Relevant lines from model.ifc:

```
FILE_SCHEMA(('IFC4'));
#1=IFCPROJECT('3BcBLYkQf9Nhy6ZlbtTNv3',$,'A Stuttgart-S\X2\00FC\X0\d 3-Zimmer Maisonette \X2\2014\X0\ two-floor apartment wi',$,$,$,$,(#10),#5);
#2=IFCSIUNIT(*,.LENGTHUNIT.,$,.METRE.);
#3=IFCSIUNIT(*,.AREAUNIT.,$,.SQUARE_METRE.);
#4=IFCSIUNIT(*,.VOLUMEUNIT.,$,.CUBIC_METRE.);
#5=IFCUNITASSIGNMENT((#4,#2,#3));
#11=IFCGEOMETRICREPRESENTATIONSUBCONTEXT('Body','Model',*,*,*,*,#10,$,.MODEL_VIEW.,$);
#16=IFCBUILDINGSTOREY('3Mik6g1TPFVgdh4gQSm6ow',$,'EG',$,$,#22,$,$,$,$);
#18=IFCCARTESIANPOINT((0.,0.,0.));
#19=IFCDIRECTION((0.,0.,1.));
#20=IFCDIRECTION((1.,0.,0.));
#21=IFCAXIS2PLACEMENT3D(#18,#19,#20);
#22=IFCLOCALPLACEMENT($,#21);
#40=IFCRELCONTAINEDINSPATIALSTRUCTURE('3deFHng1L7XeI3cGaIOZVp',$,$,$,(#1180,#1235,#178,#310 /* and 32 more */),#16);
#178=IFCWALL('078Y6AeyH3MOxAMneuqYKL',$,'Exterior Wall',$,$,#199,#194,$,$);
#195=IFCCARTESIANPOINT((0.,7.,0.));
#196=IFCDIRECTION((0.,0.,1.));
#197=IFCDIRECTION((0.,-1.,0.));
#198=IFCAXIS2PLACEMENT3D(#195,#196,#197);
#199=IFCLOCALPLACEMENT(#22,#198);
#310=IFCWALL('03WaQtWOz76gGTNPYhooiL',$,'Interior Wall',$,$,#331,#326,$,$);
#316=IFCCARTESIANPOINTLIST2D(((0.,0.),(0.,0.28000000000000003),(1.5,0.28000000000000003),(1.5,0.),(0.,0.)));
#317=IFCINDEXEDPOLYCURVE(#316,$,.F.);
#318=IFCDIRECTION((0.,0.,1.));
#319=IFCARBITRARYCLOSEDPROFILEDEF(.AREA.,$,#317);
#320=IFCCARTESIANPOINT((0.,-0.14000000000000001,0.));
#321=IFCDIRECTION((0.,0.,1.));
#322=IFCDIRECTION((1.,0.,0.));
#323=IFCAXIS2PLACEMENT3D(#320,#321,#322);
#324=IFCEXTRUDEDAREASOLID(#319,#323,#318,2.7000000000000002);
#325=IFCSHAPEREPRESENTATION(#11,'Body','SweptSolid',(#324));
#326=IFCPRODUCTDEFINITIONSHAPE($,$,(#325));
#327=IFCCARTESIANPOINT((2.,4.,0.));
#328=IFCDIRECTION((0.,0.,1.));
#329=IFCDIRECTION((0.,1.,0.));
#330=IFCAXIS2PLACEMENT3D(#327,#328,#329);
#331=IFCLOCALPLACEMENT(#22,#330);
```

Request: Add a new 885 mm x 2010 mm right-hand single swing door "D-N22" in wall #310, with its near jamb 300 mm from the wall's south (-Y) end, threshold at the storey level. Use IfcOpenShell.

```python
import numpy as np
import ifcopenshell
import ifcopenshell.api.feature
import ifcopenshell.api.geometry
import ifcopenshell.api.root
import ifcopenshell.api.spatial
import ifcopenshell.geom
import ifcopenshell.util.element
import ifcopenshell.util.placement
import ifcopenshell.util.representation
import ifcopenshell.util.shape
import ifcopenshell.util.unit

model = ifcopenshell.open("model.ifc")
unit_scale = ifcopenshell.util.unit.calculate_unit_scale(model)
settings = ifcopenshell.geom.settings()


def volume(element):
    """Net volume in cubic metres, openings subtracted."""
    shape = ifcopenshell.geom.create_shape(settings, element)
    return ifcopenshell.util.shape.get_volume(shape.geometry)


wall = model.by_guid("03WaQtWOz76gGTNPYhooiL")
storey = ifcopenshell.util.element.get_container(wall, ifc_class="IfcBuildingStorey")
context = ifcopenshell.util.representation.get_context(model, "Model", "Body", "MODEL_VIEW")
before = volume(wall)

width, height, from_end, sill = 0.885, 2.01, 0.3, 0.0  # metres

# The wall runs along its own X axis, and the end named is its -X end.
wall_shape = ifcopenshell.geom.create_shape(settings, wall)
x, y, z = ifcopenshell.util.shape.get_vertices(wall_shape.geometry).T
start = x.min() + from_end
face, thickness = float(y.min()), float(y.max() - y.min())
wall_matrix = ifcopenshell.util.placement.get_local_placement(wall.ObjectPlacement)
level = ifcopenshell.util.placement.get_local_placement(storey.ObjectPlacement)[2, 3]


def in_wall(x, y):
    """Placement at x, y metres in the wall's axes, at sill height."""
    matrix = wall_matrix.copy()
    matrix[:, 3] = wall_matrix @ np.array([x / unit_scale, y / unit_scale, 0.0, 1.0])
    matrix[2, 3] = level + sill / unit_scale
    return matrix


# Opening: a box that overshoots both wall faces by 50 mm.
opening = ifcopenshell.api.root.create_entity(model, ifc_class="IfcOpeningElement", predefined_type="OPENING")
box = ifcopenshell.api.geometry.add_wall_representation(
    model, context=context, length=width, height=height, thickness=thickness + 0.1
)
ifcopenshell.api.geometry.assign_representation(model, product=opening, representation=box)
ifcopenshell.api.geometry.edit_object_placement(model, product=opening, matrix=in_wall(start, face - 0.05), is_si=False)
ifcopenshell.api.feature.add_feature(model, feature=opening, element=wall)

door = ifcopenshell.api.root.create_entity(model, ifc_class="IfcDoor", name="D-N22", predefined_type="DOOR")
door.OverallWidth, door.OverallHeight = width / unit_scale, height / unit_scale
door.OperationType = "SINGLE_SWING_RIGHT"
body = ifcopenshell.api.geometry.add_door_representation(
    model,
    context=context,
    overall_width=door.OverallWidth,
    overall_height=door.OverallHeight,
    operation_type="SINGLE_SWING_RIGHT",
    lining_properties={"LiningDepth": thickness / unit_scale, "ThresholdDepth": thickness / unit_scale},
)
ifcopenshell.api.geometry.assign_representation(model, product=door, representation=body)
ifcopenshell.api.spatial.assign_container(model, products=[door], relating_structure=storey)
ifcopenshell.api.feature.add_filling(model, opening=opening, element=door)

# The lining spans the wall, so the door starts at the wall face.
ifcopenshell.api.geometry.edit_object_placement(model, product=door, matrix=in_wall(start, face), is_si=False)

after = volume(wall)

print(f"wall volume {before:.3f} -> {after:.3f} m3")

model.write("model_edited.ifc")
```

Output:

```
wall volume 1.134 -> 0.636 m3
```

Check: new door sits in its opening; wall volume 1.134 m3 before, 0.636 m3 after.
